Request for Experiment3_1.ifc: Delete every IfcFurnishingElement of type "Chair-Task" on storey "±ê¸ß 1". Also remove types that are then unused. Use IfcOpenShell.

First a look at what the model holds.

```python
import ifcopenshell
import ifcopenshell.util.element

model = ifcopenshell.open("Experiment3_1.ifc")
print(model.schema)
storey = next(s for s in model.by_type("IfcBuildingStorey") if s.Name == "±ê¸ß 1")
furniture = [e for e in ifcopenshell.util.element.get_decomposition(storey) if e.is_a("IfcFurnishingElement")]
seen = {}
for e in furniture:
    element_type = ifcopenshell.util.element.get_type(e)
    name = element_type.Name if element_type not in (None, e) else None
    seen[name] = seen.get(name, 0) + 1
for name, count in sorted(seen.items(), key=str):
    print(count, "x", name)
```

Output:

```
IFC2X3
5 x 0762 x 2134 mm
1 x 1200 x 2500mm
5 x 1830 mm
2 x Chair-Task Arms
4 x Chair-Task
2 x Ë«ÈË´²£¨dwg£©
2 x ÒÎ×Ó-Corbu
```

```python
import ifcopenshell
import ifcopenshell.api.root
import ifcopenshell.util.element

model = ifcopenshell.open("Experiment3_1.ifc")

storey = next(s for s in model.by_type("IfcBuildingStorey") if s.Name == "±ê¸ß 1")
furniture = [e for e in ifcopenshell.util.element.get_decomposition(storey) if e.is_a("IfcFurnishingElement")]
targets = [e for e in furniture if (t := ifcopenshell.util.element.get_type(e)) not in (None, e) and t.Name == "Chair-Task"]
types = {ifcopenshell.util.element.get_type(e) for e in targets} - {None, *targets}

for e in targets:
    ifcopenshell.api.root.remove_product(model, product=e)
print(len(targets), "removed")

unused = [t for t in types if not ifcopenshell.util.element.get_types(t)]
for t in unused:
    ifcopenshell.api.root.remove_product(model, product=t)
print(len(unused), "unused types removed")

model.write("Experiment3_1-out.ifc")
```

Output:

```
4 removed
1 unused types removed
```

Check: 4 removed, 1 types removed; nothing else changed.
